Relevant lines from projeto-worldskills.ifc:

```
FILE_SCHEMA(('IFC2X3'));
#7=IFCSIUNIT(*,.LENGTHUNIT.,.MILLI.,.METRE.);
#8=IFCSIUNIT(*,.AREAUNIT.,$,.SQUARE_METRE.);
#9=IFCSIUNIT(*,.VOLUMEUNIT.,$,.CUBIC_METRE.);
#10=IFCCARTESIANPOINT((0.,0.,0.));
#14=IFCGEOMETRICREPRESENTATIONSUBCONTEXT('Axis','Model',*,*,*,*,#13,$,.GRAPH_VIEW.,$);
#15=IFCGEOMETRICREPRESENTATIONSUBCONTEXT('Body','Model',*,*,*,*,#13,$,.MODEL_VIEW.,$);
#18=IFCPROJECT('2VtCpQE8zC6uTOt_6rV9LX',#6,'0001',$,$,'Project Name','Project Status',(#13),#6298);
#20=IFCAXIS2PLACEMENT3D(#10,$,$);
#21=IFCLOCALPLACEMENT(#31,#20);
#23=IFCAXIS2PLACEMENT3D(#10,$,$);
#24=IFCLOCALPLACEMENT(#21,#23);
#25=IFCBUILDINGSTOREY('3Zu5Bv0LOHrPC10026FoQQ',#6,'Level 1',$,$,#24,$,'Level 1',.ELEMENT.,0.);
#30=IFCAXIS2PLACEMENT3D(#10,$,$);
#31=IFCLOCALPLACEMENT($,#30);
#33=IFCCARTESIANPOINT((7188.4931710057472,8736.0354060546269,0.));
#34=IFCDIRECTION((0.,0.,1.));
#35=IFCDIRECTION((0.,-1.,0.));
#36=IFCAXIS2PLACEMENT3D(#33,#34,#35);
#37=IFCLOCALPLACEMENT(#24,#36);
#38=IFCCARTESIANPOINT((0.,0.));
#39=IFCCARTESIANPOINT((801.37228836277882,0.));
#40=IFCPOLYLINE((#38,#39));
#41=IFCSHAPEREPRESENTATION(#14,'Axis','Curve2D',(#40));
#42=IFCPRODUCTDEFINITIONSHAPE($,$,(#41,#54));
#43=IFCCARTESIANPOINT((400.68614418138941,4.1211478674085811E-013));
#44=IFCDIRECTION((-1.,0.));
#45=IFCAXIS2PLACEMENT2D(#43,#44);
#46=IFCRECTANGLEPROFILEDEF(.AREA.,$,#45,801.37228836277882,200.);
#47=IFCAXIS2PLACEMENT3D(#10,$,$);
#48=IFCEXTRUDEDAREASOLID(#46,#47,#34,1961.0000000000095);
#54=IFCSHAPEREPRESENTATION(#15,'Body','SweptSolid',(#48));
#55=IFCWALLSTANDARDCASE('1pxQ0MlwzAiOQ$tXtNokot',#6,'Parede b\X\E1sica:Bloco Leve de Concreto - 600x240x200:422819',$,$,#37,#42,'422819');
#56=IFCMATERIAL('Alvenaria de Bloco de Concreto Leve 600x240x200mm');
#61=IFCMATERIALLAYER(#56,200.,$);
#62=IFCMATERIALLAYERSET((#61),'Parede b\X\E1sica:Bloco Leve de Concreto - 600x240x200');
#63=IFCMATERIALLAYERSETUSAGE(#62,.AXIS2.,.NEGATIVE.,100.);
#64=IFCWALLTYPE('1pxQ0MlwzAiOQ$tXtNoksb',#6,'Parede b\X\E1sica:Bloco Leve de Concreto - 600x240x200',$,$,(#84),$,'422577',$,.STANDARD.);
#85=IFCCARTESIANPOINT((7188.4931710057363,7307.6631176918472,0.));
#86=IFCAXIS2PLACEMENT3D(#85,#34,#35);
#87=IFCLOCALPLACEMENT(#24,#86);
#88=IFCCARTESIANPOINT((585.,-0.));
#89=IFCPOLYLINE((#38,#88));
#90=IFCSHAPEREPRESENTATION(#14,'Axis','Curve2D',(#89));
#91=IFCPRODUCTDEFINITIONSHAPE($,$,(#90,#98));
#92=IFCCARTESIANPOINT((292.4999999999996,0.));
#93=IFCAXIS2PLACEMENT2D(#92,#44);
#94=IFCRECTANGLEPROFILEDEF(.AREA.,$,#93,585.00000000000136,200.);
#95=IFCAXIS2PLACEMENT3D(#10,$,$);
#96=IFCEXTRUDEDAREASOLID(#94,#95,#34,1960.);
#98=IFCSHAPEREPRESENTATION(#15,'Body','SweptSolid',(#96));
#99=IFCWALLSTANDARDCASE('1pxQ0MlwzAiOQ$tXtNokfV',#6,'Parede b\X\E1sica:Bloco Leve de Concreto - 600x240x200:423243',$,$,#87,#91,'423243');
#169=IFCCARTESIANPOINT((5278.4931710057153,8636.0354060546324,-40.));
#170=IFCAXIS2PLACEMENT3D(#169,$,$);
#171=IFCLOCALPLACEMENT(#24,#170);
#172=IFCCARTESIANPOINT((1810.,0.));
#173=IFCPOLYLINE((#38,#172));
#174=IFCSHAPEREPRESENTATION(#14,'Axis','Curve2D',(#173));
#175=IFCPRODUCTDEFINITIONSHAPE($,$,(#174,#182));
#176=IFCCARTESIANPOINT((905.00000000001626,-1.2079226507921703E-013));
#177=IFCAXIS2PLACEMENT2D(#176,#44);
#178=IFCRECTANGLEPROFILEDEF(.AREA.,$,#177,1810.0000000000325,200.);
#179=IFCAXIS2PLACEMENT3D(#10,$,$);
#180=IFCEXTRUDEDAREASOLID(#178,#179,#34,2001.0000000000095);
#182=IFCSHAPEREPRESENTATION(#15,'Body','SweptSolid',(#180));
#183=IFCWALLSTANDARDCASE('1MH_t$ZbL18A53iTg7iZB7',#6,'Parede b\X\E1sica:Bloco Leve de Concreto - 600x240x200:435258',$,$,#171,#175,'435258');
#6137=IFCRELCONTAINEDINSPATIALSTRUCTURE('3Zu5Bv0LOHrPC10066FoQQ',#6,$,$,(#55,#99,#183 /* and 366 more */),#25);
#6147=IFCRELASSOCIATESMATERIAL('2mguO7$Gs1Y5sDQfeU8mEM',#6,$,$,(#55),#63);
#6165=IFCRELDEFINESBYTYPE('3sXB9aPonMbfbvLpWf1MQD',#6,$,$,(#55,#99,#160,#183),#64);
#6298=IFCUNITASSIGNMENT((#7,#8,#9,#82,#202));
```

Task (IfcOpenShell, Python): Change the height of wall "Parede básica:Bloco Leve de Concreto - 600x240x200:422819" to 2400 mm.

```python
import ifcopenshell
import ifcopenshell.geom
import ifcopenshell.util.representation
import ifcopenshell.util.shape
import ifcopenshell.util.unit

model = ifcopenshell.open("projeto-worldskills.ifc")
unit_scale = ifcopenshell.util.unit.calculate_unit_scale(model)
settings = ifcopenshell.geom.settings()


def volume(element):
    """Net volume in cubic metres, openings subtracted."""
    shape = ifcopenshell.geom.create_shape(settings, element)
    return ifcopenshell.util.shape.get_volume(shape.geometry)


wall = model.by_guid("1pxQ0MlwzAiOQ$tXtNokot")
before = volume(wall)

body = ifcopenshell.util.representation.get_representation(wall, "Model", "Body")
solid = body.Items[0]
old_height = solid.Depth
solid.Depth = 2.4 / unit_scale
after = volume(wall)

print(f"height {old_height:g} -> {solid.Depth:g}, volume {before:.3f} -> {after:.3f} m3")

model.write("projeto-worldskills-out.ifc")
```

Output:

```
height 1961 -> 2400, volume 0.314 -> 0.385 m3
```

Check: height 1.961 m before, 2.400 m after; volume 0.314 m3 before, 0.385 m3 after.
